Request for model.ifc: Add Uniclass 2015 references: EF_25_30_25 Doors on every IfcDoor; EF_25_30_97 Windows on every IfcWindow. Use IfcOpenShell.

First a look at what the model holds.

```python
import ifcopenshell

model = ifcopenshell.open("model.ifc")
print(model.schema)
print("classifications:", [c.Name for c in model.by_type("IfcClassification")])
for ifc_class in ("IfcDoor", "IfcRoof", "IfcStair", "IfcWall", "IfcWindow"):
    print(ifc_class, len(model.by_type(ifc_class)))
```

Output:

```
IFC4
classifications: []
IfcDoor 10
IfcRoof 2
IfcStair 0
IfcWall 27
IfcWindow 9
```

```python
import ifcopenshell
import ifcopenshell.api.classification

model = ifcopenshell.open("model.ifc")

system = ifcopenshell.api.classification.add_classification(model, classification="Uniclass 2015")

codes = {
    "IfcDoor": ("EF_25_30_25", "Doors"),
    "IfcWindow": ("EF_25_30_97", "Windows"),
}
for ifc_class, (code, name) in codes.items():
    products = model.by_type(ifc_class)
    ifcopenshell.api.classification.add_reference(
        model, products=products, classification=system, identification=code, name=name
    )
    print(code, len(products))

model.write("model_v2.ifc")
```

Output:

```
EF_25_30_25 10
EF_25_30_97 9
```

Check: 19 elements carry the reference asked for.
